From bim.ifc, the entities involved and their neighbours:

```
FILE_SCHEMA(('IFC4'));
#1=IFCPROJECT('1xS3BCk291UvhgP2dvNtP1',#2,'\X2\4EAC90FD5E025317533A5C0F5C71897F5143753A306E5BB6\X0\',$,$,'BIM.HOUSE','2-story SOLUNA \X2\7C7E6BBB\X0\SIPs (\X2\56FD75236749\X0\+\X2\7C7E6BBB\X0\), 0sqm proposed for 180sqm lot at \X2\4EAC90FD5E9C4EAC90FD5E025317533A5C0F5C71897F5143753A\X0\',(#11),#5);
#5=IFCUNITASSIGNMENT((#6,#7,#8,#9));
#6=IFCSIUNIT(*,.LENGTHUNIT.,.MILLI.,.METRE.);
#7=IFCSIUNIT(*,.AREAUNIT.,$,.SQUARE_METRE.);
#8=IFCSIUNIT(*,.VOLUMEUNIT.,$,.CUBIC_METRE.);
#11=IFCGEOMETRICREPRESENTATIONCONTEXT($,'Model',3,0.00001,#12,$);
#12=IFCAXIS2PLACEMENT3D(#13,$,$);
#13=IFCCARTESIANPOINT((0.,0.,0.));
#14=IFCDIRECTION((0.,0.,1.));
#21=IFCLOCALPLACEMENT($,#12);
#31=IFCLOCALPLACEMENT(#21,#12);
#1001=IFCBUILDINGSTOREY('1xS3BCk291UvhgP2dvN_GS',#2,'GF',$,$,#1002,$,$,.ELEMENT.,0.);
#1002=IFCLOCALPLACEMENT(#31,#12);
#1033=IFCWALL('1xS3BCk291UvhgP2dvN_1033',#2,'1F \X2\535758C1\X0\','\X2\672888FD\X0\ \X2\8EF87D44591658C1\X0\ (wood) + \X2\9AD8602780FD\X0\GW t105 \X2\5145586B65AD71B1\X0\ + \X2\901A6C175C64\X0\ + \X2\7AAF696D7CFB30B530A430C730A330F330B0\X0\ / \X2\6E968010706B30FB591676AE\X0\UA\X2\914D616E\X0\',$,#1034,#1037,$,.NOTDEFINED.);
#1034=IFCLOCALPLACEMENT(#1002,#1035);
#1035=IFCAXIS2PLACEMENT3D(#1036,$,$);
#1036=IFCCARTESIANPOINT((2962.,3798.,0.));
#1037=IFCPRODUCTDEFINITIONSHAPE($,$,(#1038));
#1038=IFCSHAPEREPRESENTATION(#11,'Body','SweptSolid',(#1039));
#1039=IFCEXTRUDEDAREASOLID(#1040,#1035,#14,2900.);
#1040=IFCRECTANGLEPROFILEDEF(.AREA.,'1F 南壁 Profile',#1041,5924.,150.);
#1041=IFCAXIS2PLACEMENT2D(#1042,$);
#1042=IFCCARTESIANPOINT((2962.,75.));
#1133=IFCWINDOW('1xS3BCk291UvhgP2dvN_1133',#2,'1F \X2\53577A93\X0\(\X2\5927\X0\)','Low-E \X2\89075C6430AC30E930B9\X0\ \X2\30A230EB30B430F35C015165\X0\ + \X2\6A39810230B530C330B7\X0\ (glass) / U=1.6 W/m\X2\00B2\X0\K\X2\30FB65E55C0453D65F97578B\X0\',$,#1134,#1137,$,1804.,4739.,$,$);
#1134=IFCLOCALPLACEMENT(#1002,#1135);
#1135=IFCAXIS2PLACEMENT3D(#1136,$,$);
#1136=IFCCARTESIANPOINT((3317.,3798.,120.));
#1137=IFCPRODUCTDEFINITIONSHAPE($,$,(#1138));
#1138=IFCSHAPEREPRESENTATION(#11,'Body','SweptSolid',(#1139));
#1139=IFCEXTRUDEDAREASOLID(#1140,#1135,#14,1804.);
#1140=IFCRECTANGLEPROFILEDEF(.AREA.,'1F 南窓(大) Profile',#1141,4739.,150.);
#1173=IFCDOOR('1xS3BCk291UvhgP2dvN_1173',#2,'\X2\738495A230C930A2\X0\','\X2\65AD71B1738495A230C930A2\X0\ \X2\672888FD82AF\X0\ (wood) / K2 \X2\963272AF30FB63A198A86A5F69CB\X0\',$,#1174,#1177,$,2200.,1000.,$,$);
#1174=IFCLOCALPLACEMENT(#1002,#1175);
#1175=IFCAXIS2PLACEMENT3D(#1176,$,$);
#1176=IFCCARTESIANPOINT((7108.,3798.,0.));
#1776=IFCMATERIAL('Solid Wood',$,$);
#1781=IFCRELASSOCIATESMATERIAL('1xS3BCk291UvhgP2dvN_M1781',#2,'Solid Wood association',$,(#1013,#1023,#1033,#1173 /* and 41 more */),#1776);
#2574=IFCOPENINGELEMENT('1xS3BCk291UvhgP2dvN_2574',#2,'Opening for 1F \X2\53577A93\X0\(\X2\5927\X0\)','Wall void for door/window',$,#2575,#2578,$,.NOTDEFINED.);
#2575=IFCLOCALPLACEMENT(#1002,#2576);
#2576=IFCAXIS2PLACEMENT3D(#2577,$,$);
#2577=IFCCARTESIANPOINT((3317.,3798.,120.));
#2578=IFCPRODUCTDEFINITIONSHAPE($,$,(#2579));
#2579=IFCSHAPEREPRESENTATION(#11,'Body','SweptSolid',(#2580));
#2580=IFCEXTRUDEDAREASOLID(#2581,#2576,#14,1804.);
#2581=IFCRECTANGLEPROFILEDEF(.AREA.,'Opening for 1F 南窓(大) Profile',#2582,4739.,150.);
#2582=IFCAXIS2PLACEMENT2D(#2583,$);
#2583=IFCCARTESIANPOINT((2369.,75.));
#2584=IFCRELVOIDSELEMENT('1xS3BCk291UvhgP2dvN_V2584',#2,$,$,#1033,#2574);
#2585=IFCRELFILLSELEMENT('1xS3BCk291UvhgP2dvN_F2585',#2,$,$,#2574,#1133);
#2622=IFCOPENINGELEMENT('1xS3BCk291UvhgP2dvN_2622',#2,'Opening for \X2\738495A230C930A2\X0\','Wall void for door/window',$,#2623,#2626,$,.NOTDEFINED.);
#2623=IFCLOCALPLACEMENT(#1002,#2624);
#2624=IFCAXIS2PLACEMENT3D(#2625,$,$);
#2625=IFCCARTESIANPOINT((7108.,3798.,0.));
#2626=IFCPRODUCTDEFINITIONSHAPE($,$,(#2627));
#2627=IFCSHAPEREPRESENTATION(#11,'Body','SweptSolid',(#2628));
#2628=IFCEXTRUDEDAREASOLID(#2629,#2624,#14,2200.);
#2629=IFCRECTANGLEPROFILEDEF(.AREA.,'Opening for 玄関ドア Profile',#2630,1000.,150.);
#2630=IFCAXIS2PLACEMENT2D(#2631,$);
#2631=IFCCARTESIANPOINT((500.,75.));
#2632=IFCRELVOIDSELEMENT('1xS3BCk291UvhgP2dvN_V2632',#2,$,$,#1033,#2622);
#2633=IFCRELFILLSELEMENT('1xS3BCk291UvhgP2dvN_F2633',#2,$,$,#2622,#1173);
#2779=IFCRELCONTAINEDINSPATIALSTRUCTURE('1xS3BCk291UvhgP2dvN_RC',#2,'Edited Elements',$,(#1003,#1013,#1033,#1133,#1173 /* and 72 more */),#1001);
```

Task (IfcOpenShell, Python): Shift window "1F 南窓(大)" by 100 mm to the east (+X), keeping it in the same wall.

```python
import ifcopenshell
import ifcopenshell.api.geometry
import ifcopenshell.util.placement
import ifcopenshell.util.unit

model = ifcopenshell.open("bim.ifc")
unit_scale = ifcopenshell.util.unit.calculate_unit_scale(model)

window = model.by_guid("1xS3BCk291UvhgP2dvN_1133")
opening = window.FillsVoids[0].RelatingOpeningElement
wall = opening.VoidsElements[0].RelatingBuildingElement

wall_matrix = ifcopenshell.util.placement.get_local_placement(wall.ObjectPlacement)
shift = wall_matrix[:3, 0] * 0.1 / unit_scale
before = ifcopenshell.util.placement.get_local_placement(window.ObjectPlacement)[:3, 3].copy()

# The window is not placed relative to its opening, so move both.
for product in (opening, window):
    matrix = ifcopenshell.util.placement.get_local_placement(product.ObjectPlacement)
    matrix[:3, 3] += shift
    ifcopenshell.api.geometry.edit_object_placement(model, product=product, matrix=matrix, is_si=False)

after = ifcopenshell.util.placement.get_local_placement(window.ObjectPlacement)[:3, 3]
print("window moved by", (after - before).round(3) + 0.0)

model.write("bim_updated.ifc")
```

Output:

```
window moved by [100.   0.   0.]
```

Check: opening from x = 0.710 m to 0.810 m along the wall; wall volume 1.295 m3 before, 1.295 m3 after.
